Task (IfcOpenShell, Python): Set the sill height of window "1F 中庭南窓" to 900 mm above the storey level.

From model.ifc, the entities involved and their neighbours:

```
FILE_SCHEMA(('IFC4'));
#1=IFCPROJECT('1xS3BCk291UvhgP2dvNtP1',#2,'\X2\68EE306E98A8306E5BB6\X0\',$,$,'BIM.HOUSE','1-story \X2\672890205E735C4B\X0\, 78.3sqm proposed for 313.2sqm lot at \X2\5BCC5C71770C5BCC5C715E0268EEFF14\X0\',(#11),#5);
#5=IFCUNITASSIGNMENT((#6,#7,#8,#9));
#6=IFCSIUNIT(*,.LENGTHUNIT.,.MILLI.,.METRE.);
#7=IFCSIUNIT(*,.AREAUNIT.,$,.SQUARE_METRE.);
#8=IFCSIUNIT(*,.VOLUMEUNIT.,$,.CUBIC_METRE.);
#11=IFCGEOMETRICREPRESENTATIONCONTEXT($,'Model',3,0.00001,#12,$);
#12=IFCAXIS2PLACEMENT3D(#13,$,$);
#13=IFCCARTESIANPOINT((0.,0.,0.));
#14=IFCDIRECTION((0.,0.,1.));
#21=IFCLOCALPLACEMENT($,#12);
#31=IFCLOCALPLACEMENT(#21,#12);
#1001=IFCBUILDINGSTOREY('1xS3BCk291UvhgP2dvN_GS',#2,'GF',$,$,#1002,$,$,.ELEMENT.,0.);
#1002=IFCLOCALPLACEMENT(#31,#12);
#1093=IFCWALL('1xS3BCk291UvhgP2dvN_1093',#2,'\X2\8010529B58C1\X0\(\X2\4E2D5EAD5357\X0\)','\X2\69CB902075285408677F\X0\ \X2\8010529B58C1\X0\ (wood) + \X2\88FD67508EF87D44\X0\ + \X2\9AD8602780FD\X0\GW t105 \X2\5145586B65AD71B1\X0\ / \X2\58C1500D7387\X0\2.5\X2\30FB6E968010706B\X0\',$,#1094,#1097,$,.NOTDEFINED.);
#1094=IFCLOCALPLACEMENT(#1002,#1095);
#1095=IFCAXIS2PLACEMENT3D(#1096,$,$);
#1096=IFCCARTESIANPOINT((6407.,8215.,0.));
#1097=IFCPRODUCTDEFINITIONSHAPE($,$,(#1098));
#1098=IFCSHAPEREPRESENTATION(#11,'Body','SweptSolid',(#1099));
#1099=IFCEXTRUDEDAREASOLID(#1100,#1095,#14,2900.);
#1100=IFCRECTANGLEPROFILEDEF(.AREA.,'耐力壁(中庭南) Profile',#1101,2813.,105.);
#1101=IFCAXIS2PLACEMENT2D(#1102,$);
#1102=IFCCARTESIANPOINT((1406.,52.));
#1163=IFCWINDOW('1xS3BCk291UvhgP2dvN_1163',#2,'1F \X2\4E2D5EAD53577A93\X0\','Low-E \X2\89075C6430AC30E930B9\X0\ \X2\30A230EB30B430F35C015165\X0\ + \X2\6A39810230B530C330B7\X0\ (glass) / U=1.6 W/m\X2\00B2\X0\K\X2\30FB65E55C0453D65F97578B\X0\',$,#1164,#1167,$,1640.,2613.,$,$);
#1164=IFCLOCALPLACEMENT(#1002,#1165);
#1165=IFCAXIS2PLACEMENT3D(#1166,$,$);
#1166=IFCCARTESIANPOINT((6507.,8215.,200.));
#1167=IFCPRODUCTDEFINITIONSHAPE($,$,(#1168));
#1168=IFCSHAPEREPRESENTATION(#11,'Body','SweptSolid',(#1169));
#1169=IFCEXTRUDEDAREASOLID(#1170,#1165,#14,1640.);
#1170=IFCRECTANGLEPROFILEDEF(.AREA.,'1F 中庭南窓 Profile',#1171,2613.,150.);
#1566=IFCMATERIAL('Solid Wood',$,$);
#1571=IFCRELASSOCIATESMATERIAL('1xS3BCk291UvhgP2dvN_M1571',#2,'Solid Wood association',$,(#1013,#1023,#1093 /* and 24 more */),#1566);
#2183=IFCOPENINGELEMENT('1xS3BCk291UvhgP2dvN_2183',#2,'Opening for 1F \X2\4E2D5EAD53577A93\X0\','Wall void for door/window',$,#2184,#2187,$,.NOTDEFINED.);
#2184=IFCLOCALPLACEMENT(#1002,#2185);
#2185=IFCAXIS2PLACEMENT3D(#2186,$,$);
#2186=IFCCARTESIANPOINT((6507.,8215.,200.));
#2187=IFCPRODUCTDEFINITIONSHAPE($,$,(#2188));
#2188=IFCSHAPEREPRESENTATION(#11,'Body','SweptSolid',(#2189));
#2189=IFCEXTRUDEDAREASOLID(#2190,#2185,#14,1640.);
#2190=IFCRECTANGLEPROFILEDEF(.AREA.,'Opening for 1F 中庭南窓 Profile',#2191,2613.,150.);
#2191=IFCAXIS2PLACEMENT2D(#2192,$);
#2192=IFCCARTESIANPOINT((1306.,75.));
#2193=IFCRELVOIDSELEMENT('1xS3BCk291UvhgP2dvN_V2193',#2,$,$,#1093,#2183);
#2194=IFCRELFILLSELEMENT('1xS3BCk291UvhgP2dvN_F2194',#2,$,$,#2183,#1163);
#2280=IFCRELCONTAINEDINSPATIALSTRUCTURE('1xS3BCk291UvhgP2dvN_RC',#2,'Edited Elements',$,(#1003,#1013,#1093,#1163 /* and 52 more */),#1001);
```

```python
import numpy as np
import ifcopenshell
import ifcopenshell.api.geometry
import ifcopenshell.geom
import ifcopenshell.util.element
import ifcopenshell.util.placement
import ifcopenshell.util.shape
import ifcopenshell.util.unit

model = ifcopenshell.open("model.ifc")
unit_scale = ifcopenshell.util.unit.calculate_unit_scale(model)

window = model.by_guid("1xS3BCk291UvhgP2dvN_1163")
opening = window.FillsVoids[0].RelatingOpeningElement
storey = ifcopenshell.util.element.get_container(window, ifc_class="IfcBuildingStorey")
level = ifcopenshell.util.placement.get_local_placement(storey.ObjectPlacement)[2, 3]

# The opening's origin need not be at the sill, so measure its lowest point.
shape = ifcopenshell.geom.create_shape(ifcopenshell.geom.settings(), opening)
bottom = ifcopenshell.util.shape.get_shape_bottom_elevation(shape, shape.geometry) / unit_scale
dz = level + 0.9 / unit_scale - bottom

shift = np.array([0.0, 0.0, dz])
# The window is not placed relative to its opening, so move both.
for product in (opening, window):
    matrix = ifcopenshell.util.placement.get_local_placement(product.ObjectPlacement)
    matrix[:3, 3] += shift
    ifcopenshell.api.geometry.edit_object_placement(model, product=product, matrix=matrix, is_si=False)

print(f"moved by {dz * unit_scale:+.3f} m")

model.write("model_rev.ifc")
```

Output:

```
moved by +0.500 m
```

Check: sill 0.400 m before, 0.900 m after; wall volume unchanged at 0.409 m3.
